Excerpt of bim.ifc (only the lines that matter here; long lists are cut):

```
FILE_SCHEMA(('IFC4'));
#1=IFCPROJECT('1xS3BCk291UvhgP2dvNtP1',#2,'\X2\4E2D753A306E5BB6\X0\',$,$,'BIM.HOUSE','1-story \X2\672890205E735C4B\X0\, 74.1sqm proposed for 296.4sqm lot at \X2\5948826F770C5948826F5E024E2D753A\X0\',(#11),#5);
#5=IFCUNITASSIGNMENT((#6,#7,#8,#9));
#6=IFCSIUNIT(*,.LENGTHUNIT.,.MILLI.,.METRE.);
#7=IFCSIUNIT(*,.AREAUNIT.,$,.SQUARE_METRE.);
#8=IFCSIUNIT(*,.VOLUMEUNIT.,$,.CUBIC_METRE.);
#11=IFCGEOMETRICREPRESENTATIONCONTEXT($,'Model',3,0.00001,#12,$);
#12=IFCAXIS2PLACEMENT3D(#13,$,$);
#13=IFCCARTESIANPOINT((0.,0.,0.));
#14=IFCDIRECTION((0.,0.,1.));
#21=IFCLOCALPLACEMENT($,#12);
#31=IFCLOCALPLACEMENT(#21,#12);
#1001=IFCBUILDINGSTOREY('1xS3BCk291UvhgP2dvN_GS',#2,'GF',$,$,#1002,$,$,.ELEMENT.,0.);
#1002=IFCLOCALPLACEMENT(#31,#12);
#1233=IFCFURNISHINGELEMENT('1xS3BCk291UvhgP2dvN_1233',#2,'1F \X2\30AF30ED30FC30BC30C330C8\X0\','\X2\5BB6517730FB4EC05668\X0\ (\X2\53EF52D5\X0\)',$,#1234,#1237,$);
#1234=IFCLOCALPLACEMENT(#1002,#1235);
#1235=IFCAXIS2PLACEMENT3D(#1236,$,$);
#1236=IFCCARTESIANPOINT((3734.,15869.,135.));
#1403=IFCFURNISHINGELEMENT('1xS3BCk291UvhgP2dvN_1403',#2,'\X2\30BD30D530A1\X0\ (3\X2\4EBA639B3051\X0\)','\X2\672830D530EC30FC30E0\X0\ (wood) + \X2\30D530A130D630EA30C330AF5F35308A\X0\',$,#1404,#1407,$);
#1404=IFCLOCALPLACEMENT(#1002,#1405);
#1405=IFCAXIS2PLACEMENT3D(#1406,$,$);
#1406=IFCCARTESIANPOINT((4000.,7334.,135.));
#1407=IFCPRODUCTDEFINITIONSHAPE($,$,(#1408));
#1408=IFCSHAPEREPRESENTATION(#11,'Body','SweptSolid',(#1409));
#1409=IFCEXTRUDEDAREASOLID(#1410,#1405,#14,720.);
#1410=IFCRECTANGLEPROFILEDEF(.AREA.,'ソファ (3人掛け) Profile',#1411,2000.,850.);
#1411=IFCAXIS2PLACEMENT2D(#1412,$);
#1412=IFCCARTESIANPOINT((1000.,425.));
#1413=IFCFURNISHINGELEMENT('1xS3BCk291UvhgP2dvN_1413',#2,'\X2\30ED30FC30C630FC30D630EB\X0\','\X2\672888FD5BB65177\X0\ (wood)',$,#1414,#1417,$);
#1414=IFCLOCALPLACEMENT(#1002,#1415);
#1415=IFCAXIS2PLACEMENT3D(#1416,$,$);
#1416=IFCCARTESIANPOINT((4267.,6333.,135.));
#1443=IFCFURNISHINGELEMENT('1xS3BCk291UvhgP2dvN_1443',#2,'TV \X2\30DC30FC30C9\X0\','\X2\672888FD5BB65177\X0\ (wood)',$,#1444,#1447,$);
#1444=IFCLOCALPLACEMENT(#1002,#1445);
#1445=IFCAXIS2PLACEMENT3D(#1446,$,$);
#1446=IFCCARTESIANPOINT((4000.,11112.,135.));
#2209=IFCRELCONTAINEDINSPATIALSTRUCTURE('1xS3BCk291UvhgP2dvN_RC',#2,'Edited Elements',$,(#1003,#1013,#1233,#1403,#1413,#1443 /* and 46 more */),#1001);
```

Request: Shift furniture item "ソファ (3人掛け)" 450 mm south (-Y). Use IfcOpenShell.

```python
import ifcopenshell
import ifcopenshell.api.geometry
import ifcopenshell.util.placement
import ifcopenshell.util.unit

model = ifcopenshell.open("bim.ifc")
unit_scale = ifcopenshell.util.unit.calculate_unit_scale(model)

item = model.by_guid("1xS3BCk291UvhgP2dvN_1403")
matrix = ifcopenshell.util.placement.get_local_placement(item.ObjectPlacement)
matrix[1, 3] -= 0.45 / unit_scale
ifcopenshell.api.geometry.edit_object_placement(model, product=item, matrix=matrix, is_si=False)

print(ifcopenshell.util.placement.get_local_placement(item.ObjectPlacement).round(3) + 0.0)

model.write("bim_edited.ifc")
```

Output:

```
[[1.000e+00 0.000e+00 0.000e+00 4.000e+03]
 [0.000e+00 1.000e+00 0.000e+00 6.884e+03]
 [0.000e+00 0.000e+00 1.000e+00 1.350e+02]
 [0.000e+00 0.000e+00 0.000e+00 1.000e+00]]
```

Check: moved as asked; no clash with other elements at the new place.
